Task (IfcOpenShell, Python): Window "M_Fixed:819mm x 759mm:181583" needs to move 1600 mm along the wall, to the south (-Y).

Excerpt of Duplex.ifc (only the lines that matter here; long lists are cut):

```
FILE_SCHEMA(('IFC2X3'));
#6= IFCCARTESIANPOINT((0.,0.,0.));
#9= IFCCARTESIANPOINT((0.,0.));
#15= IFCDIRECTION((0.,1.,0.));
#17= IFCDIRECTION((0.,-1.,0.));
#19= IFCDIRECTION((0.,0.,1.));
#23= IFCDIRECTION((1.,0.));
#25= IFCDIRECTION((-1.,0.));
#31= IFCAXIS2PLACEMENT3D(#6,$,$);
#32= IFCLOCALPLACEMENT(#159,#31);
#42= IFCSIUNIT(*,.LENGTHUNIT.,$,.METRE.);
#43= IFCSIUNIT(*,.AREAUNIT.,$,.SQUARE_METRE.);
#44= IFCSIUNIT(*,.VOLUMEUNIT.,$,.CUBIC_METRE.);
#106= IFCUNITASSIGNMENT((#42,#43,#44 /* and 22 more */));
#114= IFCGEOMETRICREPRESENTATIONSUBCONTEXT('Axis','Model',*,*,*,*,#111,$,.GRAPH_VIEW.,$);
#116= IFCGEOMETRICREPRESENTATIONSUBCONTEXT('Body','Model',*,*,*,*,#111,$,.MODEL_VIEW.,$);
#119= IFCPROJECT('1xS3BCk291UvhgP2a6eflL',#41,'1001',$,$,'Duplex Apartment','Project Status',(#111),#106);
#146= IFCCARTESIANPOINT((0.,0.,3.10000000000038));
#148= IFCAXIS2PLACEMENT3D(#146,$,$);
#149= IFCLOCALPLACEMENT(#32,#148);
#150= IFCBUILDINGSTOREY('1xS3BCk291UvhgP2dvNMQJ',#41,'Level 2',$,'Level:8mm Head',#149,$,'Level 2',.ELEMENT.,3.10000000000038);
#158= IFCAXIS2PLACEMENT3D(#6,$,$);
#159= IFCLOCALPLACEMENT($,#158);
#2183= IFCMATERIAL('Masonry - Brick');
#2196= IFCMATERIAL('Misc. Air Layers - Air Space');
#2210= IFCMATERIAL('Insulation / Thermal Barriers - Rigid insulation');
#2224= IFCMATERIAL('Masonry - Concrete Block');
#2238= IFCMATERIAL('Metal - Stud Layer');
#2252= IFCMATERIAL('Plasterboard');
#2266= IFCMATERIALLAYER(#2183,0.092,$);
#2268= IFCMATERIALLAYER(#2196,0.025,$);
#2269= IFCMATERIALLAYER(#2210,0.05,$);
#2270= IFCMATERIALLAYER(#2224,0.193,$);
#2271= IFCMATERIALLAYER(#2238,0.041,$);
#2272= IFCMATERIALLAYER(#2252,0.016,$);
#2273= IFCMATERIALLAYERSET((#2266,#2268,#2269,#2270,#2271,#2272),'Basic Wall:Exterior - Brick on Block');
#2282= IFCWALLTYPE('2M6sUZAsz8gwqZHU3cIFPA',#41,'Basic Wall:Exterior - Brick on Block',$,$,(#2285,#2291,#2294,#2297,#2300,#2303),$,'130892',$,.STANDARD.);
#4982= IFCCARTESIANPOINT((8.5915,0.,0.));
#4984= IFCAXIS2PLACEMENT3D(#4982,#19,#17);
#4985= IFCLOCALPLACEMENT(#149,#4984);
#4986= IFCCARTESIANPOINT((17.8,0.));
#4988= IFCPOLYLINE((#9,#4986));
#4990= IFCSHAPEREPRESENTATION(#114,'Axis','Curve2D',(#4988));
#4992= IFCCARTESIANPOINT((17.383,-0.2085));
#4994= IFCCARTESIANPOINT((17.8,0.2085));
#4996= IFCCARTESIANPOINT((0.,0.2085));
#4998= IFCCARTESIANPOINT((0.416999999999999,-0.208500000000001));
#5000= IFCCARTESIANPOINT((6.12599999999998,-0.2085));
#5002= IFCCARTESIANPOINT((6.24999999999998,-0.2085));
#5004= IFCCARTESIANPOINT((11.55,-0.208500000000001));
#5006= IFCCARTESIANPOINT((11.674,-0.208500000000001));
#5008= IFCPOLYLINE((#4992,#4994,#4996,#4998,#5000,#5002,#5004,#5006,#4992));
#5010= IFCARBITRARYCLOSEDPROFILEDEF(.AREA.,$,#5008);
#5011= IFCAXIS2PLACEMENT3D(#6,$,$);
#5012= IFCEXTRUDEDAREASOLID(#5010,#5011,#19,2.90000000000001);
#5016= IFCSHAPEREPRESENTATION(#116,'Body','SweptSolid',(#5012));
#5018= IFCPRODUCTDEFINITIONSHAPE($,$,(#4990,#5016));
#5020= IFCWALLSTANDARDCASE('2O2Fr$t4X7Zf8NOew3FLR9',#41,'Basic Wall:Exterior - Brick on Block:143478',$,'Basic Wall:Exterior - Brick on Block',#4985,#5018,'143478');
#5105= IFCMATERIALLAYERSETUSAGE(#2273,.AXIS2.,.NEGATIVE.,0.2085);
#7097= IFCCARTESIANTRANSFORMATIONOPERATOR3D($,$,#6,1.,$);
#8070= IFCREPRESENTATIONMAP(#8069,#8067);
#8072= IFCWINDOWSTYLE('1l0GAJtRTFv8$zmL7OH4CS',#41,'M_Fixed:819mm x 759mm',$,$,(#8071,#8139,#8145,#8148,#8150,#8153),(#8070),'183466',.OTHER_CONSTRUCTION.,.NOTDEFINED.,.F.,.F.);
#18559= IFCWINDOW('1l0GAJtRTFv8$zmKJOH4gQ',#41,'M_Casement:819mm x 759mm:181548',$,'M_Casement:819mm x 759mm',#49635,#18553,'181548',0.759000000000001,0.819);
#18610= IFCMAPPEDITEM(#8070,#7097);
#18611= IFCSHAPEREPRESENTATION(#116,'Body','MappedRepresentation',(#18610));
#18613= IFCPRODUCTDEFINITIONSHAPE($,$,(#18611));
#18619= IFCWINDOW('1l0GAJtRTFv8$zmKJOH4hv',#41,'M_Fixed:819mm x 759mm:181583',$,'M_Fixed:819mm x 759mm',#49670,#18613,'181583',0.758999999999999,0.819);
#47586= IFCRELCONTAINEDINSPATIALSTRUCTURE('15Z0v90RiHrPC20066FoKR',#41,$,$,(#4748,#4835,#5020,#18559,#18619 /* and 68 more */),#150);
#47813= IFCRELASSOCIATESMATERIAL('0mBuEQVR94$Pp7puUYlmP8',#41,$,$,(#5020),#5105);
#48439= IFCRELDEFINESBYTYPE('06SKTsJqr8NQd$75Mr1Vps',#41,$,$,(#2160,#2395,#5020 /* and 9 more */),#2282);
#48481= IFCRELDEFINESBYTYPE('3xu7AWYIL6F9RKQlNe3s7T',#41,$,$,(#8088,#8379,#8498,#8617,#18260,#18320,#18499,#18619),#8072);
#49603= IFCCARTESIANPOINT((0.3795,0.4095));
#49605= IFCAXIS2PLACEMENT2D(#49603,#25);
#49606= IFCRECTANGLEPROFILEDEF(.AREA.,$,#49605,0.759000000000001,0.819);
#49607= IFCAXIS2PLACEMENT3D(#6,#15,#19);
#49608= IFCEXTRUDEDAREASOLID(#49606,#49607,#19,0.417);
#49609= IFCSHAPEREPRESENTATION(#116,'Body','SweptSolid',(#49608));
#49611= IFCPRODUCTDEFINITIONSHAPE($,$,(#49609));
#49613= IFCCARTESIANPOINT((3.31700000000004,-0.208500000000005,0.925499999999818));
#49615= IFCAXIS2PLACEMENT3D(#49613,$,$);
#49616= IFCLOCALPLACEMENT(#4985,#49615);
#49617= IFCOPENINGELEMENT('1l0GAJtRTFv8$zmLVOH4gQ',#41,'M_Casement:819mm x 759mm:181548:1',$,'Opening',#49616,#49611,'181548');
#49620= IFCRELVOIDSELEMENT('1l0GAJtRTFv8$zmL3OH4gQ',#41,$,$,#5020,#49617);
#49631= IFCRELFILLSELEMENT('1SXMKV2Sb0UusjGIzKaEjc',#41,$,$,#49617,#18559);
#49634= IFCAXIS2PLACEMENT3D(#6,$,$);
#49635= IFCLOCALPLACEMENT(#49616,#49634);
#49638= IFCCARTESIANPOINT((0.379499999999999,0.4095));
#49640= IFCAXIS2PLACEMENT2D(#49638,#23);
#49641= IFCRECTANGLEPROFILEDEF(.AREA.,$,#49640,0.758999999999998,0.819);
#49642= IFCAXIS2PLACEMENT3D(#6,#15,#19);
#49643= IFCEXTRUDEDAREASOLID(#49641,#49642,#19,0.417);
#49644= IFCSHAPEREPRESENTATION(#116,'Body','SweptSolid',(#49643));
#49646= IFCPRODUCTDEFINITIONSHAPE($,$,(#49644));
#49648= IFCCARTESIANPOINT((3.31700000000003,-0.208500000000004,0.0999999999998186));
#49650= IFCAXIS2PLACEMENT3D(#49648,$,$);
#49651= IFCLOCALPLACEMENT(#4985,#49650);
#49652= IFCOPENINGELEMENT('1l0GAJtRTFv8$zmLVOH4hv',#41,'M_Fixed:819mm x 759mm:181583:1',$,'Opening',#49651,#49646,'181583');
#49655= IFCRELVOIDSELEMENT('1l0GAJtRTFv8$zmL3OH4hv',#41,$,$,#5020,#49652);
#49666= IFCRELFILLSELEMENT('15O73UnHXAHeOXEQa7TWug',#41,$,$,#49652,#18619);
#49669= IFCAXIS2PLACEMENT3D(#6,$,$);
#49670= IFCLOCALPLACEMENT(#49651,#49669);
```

```python
import ifcopenshell
import ifcopenshell.api.geometry
import ifcopenshell.util.placement
import ifcopenshell.util.unit

model = ifcopenshell.open("Duplex.ifc")
unit_scale = ifcopenshell.util.unit.calculate_unit_scale(model)

window = model.by_guid("1l0GAJtRTFv8$zmKJOH4hv")
opening = window.FillsVoids[0].RelatingOpeningElement
wall = opening.VoidsElements[0].RelatingBuildingElement

wall_matrix = ifcopenshell.util.placement.get_local_placement(wall.ObjectPlacement)
shift = wall_matrix[:3, 0] * 1.6 / unit_scale
before = ifcopenshell.util.placement.get_local_placement(window.ObjectPlacement)[:3, 3].copy()

# The window is placed relative to its opening, so it follows when the opening moves.
matrix = ifcopenshell.util.placement.get_local_placement(opening.ObjectPlacement)
matrix[:3, 3] += shift
ifcopenshell.api.geometry.edit_object_placement(
    model, product=opening, matrix=matrix, is_si=False, should_transform_children=True
)

after = ifcopenshell.util.placement.get_local_placement(window.ObjectPlacement)[:3, 3]
print("window moved by", (after - before).round(3) + 0.0)

model.write("Duplex_updated.ifc")
```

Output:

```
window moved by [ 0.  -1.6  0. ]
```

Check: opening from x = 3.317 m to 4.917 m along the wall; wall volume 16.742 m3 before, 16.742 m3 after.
